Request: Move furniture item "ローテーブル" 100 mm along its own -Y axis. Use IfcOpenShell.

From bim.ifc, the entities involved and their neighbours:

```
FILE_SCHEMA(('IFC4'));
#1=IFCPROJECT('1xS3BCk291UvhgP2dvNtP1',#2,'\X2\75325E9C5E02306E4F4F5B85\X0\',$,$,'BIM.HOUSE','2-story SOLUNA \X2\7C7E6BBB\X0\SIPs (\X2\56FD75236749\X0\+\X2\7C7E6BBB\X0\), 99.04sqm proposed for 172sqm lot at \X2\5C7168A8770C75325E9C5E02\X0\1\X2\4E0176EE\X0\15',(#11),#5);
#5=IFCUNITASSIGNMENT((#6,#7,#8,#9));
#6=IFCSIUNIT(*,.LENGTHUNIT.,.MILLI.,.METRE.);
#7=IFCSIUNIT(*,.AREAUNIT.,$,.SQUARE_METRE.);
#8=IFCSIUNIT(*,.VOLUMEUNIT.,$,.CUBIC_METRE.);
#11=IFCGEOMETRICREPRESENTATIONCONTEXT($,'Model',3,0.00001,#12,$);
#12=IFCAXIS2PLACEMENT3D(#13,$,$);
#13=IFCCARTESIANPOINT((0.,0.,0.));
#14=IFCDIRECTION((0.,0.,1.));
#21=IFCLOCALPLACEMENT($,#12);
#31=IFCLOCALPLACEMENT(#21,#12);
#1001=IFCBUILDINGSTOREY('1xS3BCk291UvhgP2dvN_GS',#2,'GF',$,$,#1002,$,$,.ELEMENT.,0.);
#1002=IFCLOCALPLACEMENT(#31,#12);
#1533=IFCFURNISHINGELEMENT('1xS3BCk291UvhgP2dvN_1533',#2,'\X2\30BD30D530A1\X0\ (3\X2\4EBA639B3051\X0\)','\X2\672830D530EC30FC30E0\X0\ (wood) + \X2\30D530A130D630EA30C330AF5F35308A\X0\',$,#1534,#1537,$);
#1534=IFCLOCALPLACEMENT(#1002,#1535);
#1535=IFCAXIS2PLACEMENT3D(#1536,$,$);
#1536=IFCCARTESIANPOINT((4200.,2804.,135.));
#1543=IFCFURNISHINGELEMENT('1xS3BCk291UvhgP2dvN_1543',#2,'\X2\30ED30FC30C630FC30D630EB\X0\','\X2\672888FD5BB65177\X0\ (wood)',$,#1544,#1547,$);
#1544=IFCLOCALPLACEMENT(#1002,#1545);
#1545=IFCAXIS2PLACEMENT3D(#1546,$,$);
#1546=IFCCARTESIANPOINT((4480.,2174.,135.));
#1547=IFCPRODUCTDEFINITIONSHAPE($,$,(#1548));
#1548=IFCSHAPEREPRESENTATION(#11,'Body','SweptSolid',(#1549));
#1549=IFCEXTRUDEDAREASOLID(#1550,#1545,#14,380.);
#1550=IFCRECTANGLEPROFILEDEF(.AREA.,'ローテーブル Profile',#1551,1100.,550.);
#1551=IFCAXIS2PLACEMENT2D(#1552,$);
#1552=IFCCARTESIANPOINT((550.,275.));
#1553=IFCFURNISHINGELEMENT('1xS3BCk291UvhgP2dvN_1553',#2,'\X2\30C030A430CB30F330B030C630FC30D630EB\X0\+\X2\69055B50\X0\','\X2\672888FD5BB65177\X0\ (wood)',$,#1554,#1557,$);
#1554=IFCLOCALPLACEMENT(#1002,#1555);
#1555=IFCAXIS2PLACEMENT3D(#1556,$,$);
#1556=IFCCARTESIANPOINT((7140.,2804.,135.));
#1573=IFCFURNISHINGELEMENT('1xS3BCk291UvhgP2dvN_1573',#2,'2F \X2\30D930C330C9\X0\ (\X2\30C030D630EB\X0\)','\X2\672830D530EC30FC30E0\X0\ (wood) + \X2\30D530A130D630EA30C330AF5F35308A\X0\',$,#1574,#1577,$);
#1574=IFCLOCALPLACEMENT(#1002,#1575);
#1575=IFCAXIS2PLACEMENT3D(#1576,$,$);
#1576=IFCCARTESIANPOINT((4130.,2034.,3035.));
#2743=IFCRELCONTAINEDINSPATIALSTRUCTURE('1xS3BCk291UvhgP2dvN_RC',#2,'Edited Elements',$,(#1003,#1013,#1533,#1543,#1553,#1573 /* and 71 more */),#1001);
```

```python
import ifcopenshell
import ifcopenshell.api.geometry
import ifcopenshell.util.placement
import ifcopenshell.util.unit

model = ifcopenshell.open("bim.ifc")
unit_scale = ifcopenshell.util.unit.calculate_unit_scale(model)

item = model.by_guid("1xS3BCk291UvhgP2dvN_1543")
matrix = ifcopenshell.util.placement.get_local_placement(item.ObjectPlacement)
matrix[:3, 3] -= matrix[:3, 1] * 0.1 / unit_scale
ifcopenshell.api.geometry.edit_object_placement(model, product=item, matrix=matrix, is_si=False)

print(ifcopenshell.util.placement.get_local_placement(item.ObjectPlacement).round(3) + 0.0)

model.write("bim-out.ifc")
```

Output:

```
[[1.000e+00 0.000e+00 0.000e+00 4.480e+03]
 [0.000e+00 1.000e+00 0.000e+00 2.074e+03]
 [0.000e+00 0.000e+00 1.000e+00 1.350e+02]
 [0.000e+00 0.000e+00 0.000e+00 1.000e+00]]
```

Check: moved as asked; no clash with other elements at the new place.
